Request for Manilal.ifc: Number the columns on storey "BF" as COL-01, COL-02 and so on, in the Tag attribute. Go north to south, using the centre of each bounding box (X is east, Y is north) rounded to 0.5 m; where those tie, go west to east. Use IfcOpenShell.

First a look at what the model holds.

```python
import ifcopenshell
import ifcopenshell.util.element
import ifcopenshell.util.placement

model = ifcopenshell.open("Manilal.ifc")
print(model.schema)
storey = next(s for s in model.by_type("IfcBuildingStorey") if s.Name == "BF")
columns = [e for e in ifcopenshell.util.element.get_decomposition(storey) if e.is_a("IfcColumn")]
for e in sorted(columns, key=lambda e: e.id()):
    origin = ifcopenshell.util.placement.get_local_placement(e.ObjectPlacement)[:3, 3]
    print(e.id(), e.Tag, e.Name, origin.round(2) + 0.0, sep=" | ")
```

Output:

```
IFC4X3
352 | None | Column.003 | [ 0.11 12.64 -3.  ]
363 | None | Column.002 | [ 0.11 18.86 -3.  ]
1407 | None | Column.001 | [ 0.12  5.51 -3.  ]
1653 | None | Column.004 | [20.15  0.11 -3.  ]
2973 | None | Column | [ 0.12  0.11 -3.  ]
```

```python
import ifcopenshell
import ifcopenshell.geom
import ifcopenshell.util.element
import ifcopenshell.util.shape

model = ifcopenshell.open("Manilal.ifc")
settings = ifcopenshell.geom.settings()
settings.set("use-world-coords", True)


def centre(element):
    shape = ifcopenshell.geom.create_shape(settings, element)
    return ifcopenshell.util.shape.get_bbox_centroid(shape.geometry)


storey = next(s for s in model.by_type("IfcBuildingStorey") if s.Name == "BF")
columns = [e for e in ifcopenshell.util.element.get_decomposition(storey) if e.is_a("IfcColumn")]

# Insertion points can sit at a corner or the storey origin, so sort by the geometry (in metres).
centres = {e: centre(e) for e in columns}
columns.sort(key=lambda e: (-round(centres[e][1] / 0.5), centres[e][0]))

for i, e in enumerate(columns, start=1):
    number = f"COL-{i:02d}"
    e.Tag = number
    print(e.id(), number)

model.write("Manilal_rev.ifc")
```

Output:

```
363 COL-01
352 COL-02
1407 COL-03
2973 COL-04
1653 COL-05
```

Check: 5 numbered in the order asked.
